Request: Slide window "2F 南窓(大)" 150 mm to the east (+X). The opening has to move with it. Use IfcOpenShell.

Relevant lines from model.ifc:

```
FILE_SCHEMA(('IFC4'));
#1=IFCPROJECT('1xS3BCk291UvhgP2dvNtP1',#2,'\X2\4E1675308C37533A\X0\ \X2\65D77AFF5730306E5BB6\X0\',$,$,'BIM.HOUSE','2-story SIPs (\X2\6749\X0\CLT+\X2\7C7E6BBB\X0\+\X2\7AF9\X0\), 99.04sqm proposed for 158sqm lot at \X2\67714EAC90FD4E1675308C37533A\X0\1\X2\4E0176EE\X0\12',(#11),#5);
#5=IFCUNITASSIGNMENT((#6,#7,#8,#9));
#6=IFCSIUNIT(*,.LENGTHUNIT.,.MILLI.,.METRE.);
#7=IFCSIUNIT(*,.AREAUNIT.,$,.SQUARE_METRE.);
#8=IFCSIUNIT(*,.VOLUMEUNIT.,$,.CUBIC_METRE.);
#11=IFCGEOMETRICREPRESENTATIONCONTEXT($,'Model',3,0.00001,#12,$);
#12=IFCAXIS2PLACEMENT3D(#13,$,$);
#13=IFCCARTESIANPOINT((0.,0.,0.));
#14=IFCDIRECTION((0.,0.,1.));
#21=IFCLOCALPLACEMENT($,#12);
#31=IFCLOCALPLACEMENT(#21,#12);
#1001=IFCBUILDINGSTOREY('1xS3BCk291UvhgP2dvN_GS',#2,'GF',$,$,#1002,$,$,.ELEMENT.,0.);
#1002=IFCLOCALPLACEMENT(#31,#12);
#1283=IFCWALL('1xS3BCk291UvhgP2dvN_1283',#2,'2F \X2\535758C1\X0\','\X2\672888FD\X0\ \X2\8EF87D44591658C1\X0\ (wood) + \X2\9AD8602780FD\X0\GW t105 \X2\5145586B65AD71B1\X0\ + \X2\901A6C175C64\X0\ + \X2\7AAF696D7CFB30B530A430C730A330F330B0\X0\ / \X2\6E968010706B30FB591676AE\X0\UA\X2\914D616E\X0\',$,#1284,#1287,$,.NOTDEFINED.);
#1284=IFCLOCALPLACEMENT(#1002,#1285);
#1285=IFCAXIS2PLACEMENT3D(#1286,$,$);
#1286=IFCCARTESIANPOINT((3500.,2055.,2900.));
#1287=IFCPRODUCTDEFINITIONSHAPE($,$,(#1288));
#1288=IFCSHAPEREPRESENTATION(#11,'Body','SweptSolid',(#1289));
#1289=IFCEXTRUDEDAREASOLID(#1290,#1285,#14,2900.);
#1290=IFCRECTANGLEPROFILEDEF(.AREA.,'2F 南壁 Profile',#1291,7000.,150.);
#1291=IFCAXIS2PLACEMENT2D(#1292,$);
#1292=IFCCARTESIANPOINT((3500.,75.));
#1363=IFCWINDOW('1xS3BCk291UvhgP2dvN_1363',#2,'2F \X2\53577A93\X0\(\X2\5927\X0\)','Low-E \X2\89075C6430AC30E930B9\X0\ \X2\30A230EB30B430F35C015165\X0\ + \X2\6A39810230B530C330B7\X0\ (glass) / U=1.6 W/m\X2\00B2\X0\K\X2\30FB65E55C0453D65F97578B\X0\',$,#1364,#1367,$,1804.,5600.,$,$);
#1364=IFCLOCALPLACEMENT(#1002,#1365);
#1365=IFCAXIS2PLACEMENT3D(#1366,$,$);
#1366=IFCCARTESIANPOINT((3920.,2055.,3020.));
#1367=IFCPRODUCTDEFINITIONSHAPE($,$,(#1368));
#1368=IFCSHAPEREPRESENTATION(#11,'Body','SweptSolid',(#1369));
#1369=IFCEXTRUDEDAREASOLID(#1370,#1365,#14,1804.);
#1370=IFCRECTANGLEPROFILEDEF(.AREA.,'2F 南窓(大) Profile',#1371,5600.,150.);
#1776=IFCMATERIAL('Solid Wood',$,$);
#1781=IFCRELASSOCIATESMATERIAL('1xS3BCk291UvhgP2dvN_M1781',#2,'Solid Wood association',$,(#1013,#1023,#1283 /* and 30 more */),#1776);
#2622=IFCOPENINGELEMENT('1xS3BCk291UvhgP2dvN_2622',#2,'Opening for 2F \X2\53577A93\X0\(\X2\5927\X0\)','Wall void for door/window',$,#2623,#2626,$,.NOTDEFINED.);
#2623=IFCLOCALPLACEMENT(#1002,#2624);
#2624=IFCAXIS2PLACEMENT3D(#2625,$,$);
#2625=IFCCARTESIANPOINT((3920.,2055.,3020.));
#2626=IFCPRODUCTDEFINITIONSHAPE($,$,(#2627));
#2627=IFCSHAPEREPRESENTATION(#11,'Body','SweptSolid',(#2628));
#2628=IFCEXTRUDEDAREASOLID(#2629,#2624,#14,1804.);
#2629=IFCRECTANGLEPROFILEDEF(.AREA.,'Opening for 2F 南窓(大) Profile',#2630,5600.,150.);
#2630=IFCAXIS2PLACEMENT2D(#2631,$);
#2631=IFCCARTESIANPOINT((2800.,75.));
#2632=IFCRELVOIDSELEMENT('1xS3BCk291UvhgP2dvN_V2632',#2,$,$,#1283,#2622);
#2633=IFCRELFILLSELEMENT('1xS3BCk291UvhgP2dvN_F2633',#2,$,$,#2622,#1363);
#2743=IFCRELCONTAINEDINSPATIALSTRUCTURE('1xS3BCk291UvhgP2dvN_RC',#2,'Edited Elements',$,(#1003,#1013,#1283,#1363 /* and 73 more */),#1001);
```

```python
import ifcopenshell
import ifcopenshell.api.geometry
import ifcopenshell.util.placement
import ifcopenshell.util.unit

model = ifcopenshell.open("model.ifc")
unit_scale = ifcopenshell.util.unit.calculate_unit_scale(model)

window = model.by_guid("1xS3BCk291UvhgP2dvN_1363")
opening = window.FillsVoids[0].RelatingOpeningElement
wall = opening.VoidsElements[0].RelatingBuildingElement

wall_matrix = ifcopenshell.util.placement.get_local_placement(wall.ObjectPlacement)
shift = wall_matrix[:3, 0] * 0.15 / unit_scale
before = ifcopenshell.util.placement.get_local_placement(window.ObjectPlacement)[:3, 3].copy()

# The window is not placed relative to its opening, so move both.
for product in (opening, window):
    matrix = ifcopenshell.util.placement.get_local_placement(product.ObjectPlacement)
    matrix[:3, 3] += shift
    ifcopenshell.api.geometry.edit_object_placement(model, product=product, matrix=matrix, is_si=False)

after = ifcopenshell.util.placement.get_local_placement(window.ObjectPlacement)[:3, 3]
print("window moved by", (after - before).round(3) + 0.0)

model.write("model_rev.ifc")
```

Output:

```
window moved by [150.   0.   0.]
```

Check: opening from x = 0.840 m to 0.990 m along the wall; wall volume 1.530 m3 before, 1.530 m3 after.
